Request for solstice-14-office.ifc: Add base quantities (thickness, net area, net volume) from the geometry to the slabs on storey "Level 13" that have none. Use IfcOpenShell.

First a look at what the model holds.

```python
import ifcopenshell
import ifcopenshell.util.element
import ifcopenshell.util.unit

model = ifcopenshell.open("solstice-14-office.ifc")
print(model.schema)
for unit_type in ("LENGTHUNIT", "AREAUNIT", "VOLUMEUNIT"):
    print(unit_type, ifcopenshell.util.unit.calculate_unit_scale(model, unit_type))
storey = next(s for s in model.by_type("IfcBuildingStorey") if s.Name == "Level 13")
slabs = [e for e in ifcopenshell.util.element.get_decomposition(storey) if e.is_a("IfcSlab")]
for e in sorted(slabs, key=lambda e: e.id()):
    print(e.id(), e.is_a(), e.Name, list(ifcopenshell.util.element.get_psets(e, qtos_only=True)), sep=" | ")
```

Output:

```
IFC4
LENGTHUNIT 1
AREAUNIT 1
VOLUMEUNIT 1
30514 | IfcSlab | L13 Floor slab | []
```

```python
import ifcopenshell
import ifcopenshell.api.pset
import ifcopenshell.geom
import ifcopenshell.util.element
import ifcopenshell.util.shape
import ifcopenshell.util.unit

model = ifcopenshell.open("solstice-14-office.ifc")
unit_scale = ifcopenshell.util.unit.calculate_unit_scale(model)
area_scale = ifcopenshell.util.unit.calculate_unit_scale(model, "AREAUNIT")
volume_scale = ifcopenshell.util.unit.calculate_unit_scale(model, "VOLUMEUNIT")
settings = ifcopenshell.geom.settings()

storey = next(s for s in model.by_type("IfcBuildingStorey") if s.Name == "Level 13")
slabs = [e for e in ifcopenshell.util.element.get_decomposition(storey) if e.is_a("IfcSlab")]

for e in sorted(slabs, key=lambda e: e.id()):
    if ifcopenshell.util.element.get_psets(e, qtos_only=True, should_inherit=False):
        continue
    # Geometry comes back in metres, in the element's own axes.
    shape = ifcopenshell.geom.create_shape(settings, e)
    values = {
        "Width": ifcopenshell.util.shape.get_z(shape.geometry) / unit_scale,
        "NetArea": ifcopenshell.util.shape.get_footprint_area(shape.geometry) / area_scale,
        "NetVolume": ifcopenshell.util.shape.get_volume(shape.geometry) / volume_scale,
    }
    qto = ifcopenshell.api.pset.add_qto(model, product=e, name="Qto_SlabBaseQuantities")
    ifcopenshell.api.pset.edit_qto(model, qto=qto, properties=values)
    print(e.id(), {k: round(v, 3) for k, v in values.items()})

model.write("solstice-14-office_rev.ifc")
```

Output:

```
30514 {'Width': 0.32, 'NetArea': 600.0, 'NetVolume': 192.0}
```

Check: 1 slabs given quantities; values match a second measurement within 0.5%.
